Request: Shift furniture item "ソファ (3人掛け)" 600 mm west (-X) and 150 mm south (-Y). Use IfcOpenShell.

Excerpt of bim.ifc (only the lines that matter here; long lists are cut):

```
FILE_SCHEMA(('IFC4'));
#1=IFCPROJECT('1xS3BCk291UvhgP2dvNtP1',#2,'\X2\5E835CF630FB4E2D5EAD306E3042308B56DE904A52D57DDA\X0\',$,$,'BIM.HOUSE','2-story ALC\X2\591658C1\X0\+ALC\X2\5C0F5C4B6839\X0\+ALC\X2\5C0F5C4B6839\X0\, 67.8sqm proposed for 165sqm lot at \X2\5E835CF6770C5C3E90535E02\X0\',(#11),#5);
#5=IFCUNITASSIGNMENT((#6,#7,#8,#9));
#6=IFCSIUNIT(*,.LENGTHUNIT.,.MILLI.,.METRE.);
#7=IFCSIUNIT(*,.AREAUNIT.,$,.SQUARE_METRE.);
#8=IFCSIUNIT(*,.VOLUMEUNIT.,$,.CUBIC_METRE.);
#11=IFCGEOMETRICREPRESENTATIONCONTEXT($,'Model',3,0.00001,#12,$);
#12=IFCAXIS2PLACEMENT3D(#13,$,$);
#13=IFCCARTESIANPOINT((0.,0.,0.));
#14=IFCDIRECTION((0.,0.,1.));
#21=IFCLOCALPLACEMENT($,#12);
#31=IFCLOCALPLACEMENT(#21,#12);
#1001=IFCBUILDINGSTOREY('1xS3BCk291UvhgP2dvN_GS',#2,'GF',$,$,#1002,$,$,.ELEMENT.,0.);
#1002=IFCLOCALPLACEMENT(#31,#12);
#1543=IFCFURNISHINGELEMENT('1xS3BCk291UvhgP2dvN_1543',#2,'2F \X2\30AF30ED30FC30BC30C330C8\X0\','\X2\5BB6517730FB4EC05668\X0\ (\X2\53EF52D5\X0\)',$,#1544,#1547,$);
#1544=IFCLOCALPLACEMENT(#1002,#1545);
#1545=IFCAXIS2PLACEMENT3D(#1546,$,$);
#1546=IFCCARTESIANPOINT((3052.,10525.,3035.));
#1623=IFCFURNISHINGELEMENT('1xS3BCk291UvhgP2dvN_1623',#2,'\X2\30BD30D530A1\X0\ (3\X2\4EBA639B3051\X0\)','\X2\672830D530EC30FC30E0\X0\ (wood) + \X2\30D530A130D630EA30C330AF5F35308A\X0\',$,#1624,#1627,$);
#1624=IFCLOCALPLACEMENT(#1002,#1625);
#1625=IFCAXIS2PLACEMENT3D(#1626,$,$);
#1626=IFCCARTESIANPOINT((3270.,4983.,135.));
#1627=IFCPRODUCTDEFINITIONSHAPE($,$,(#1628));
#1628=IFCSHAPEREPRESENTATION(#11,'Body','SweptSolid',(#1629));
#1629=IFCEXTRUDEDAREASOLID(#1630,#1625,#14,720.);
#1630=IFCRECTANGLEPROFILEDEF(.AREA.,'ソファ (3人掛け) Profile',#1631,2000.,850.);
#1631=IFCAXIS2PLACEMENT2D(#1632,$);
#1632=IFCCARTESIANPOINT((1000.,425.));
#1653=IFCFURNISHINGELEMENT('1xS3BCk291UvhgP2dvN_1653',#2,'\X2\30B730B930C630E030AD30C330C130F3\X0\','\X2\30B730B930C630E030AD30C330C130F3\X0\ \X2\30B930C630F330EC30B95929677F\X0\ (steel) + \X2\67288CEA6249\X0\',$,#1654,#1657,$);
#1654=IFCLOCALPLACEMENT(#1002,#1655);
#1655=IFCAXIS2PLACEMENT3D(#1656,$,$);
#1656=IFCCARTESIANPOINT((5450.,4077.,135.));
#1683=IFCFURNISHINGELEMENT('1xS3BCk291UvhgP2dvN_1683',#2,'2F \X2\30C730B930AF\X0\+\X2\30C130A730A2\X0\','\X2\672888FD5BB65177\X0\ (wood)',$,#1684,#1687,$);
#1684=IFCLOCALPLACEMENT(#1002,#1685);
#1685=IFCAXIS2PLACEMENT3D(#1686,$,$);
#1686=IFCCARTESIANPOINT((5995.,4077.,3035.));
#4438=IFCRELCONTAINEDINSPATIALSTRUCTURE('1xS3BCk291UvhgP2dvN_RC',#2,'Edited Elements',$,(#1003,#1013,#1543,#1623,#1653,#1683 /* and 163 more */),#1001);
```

```python
import ifcopenshell
import ifcopenshell.api.geometry
import ifcopenshell.util.placement

model = ifcopenshell.open("bim.ifc")

item = model.by_guid("1xS3BCk291UvhgP2dvN_1623")
matrix = ifcopenshell.util.placement.get_local_placement(item.ObjectPlacement)
matrix[0, 3] -= 600.0
matrix[1, 3] -= 150.0
ifcopenshell.api.geometry.edit_object_placement(model, product=item, matrix=matrix, is_si=False)

print(ifcopenshell.util.placement.get_local_placement(item.ObjectPlacement).round(3) + 0.0)

model.write("bim_updated.ifc")
```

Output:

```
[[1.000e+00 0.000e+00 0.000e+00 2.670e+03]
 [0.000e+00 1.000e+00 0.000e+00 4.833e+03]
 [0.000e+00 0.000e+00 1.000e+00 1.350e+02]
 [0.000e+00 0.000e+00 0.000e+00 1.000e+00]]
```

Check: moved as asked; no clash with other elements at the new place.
